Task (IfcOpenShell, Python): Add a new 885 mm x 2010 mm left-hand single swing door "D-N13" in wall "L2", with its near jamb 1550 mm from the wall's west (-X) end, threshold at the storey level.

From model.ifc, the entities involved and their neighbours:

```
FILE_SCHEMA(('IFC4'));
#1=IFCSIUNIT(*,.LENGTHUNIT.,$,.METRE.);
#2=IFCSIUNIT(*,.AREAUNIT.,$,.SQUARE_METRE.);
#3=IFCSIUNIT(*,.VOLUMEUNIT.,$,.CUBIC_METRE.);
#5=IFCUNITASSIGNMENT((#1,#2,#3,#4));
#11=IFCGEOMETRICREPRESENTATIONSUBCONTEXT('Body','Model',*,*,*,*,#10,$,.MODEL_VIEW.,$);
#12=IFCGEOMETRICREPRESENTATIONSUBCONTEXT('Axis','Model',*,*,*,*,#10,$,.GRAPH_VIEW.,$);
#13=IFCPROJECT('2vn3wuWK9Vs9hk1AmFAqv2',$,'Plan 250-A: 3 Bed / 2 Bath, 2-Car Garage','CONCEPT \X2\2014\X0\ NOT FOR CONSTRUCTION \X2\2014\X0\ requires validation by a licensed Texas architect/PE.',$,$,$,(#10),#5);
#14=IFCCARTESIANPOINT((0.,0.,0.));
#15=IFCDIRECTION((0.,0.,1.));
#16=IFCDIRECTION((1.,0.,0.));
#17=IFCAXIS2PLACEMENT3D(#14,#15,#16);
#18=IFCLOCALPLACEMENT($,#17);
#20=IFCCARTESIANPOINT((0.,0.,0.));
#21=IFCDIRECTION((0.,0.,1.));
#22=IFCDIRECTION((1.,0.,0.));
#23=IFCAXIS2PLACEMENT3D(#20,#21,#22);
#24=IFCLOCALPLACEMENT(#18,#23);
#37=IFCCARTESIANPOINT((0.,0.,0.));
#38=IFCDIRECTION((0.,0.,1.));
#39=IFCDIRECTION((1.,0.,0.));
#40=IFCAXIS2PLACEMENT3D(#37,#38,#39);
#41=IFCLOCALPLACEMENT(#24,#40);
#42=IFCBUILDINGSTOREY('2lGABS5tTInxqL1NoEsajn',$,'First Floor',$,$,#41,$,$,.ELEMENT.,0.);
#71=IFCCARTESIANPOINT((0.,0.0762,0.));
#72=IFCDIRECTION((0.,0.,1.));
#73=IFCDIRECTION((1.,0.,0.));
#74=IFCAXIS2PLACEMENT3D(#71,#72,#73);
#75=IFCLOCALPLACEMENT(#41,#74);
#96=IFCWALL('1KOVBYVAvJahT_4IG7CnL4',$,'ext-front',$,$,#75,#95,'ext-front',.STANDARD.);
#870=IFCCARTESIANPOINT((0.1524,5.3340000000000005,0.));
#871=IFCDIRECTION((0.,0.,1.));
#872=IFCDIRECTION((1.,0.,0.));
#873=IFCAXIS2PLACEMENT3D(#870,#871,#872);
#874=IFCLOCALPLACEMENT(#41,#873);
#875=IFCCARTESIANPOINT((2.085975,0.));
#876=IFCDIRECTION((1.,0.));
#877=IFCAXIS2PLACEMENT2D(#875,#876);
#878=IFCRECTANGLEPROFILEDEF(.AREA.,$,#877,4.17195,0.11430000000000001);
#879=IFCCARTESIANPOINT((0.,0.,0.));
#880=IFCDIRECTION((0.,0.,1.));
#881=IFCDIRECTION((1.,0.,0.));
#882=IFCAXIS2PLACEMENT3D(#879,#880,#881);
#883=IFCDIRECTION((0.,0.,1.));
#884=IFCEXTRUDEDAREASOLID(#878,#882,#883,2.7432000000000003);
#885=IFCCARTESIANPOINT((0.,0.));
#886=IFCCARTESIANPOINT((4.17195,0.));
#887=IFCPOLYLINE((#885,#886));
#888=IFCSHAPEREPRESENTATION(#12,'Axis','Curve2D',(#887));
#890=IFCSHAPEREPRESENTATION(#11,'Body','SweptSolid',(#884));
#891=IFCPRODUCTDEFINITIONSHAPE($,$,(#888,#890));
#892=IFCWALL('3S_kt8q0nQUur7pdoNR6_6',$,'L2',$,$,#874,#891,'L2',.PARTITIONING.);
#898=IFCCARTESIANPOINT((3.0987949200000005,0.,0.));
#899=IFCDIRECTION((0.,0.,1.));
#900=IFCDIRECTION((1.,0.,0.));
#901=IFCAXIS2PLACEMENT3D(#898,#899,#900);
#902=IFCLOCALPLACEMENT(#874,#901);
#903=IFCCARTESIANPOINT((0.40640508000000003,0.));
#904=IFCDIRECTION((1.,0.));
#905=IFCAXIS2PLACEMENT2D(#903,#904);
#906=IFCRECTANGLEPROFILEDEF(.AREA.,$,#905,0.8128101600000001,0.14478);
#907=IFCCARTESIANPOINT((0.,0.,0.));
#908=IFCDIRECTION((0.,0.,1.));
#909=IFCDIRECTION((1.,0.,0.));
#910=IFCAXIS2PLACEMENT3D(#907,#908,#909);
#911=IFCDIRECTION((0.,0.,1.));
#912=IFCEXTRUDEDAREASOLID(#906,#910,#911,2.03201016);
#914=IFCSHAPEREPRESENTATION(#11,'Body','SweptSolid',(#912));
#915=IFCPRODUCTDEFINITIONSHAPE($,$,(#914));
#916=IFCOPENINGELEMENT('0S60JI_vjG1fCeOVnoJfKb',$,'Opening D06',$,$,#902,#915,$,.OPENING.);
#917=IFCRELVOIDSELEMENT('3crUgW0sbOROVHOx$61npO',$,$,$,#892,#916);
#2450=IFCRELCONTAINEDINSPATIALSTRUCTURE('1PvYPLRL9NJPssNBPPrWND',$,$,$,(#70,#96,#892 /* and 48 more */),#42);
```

```python
import numpy as np
import ifcopenshell
import ifcopenshell.api.feature
import ifcopenshell.api.geometry
import ifcopenshell.api.root
import ifcopenshell.api.spatial
import ifcopenshell.geom
import ifcopenshell.util.element
import ifcopenshell.util.placement
import ifcopenshell.util.representation
import ifcopenshell.util.shape
import ifcopenshell.util.unit

model = ifcopenshell.open("model.ifc")
unit_scale = ifcopenshell.util.unit.calculate_unit_scale(model)
settings = ifcopenshell.geom.settings()


def volume(element):
    """Net volume in cubic metres, openings subtracted."""
    shape = ifcopenshell.geom.create_shape(settings, element)
    return ifcopenshell.util.shape.get_volume(shape.geometry)


wall = model.by_id(892)
storey = ifcopenshell.util.element.get_container(wall, ifc_class="IfcBuildingStorey")
context = ifcopenshell.util.representation.get_context(model, "Model", "Body", "MODEL_VIEW")
before = volume(wall)

width, height, from_end, sill = 0.885, 2.01, 1.55, 0.0  # metres

# The wall runs along its own X axis, and the end named is its -X end.
wall_shape = ifcopenshell.geom.create_shape(settings, wall)
x, y, z = ifcopenshell.util.shape.get_vertices(wall_shape.geometry).T
start = x.min() + from_end
face, thickness = float(y.min()), float(y.max() - y.min())
wall_matrix = ifcopenshell.util.placement.get_local_placement(wall.ObjectPlacement)
level = ifcopenshell.util.placement.get_local_placement(storey.ObjectPlacement)[2, 3]


def in_wall(x, y):
    """Placement at x, y metres in the wall's axes, at sill height."""
    matrix = wall_matrix.copy()
    matrix[:, 3] = wall_matrix @ np.array([x / unit_scale, y / unit_scale, 0.0, 1.0])
    matrix[2, 3] = level + sill / unit_scale
    return matrix


# Opening: a box that overshoots both wall faces by 50 mm.
opening = ifcopenshell.api.root.create_entity(model, ifc_class="IfcOpeningElement", predefined_type="OPENING")
box = ifcopenshell.api.geometry.add_wall_representation(
    model, context=context, length=width, height=height, thickness=thickness + 0.1
)
ifcopenshell.api.geometry.assign_representation(model, product=opening, representation=box)
ifcopenshell.api.geometry.edit_object_placement(model, product=opening, matrix=in_wall(start, face - 0.05), is_si=False)
ifcopenshell.api.feature.add_feature(model, feature=opening, element=wall)

door = ifcopenshell.api.root.create_entity(model, ifc_class="IfcDoor", name="D-N13", predefined_type="DOOR")
door.OverallWidth, door.OverallHeight = width / unit_scale, height / unit_scale
door.OperationType = "SINGLE_SWING_LEFT"
body = ifcopenshell.api.geometry.add_door_representation(
    model,
    context=context,
    overall_width=door.OverallWidth,
    overall_height=door.OverallHeight,
    operation_type="SINGLE_SWING_LEFT",
    lining_properties={"LiningDepth": thickness / unit_scale, "ThresholdDepth": thickness / unit_scale},
)
ifcopenshell.api.geometry.assign_representation(model, product=door, representation=body)
ifcopenshell.api.spatial.assign_container(model, products=[door], relating_structure=storey)
ifcopenshell.api.feature.add_filling(model, opening=opening, element=door)

# The lining spans the wall, so the door starts at the wall face.
ifcopenshell.api.geometry.edit_object_placement(model, product=door, matrix=in_wall(start, face), is_si=False)

after = volume(wall)

print(f"wall volume {before:.3f} -> {after:.3f} m3")

model.write("model_v2.ifc")
```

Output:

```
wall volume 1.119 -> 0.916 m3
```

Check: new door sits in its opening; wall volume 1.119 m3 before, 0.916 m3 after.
